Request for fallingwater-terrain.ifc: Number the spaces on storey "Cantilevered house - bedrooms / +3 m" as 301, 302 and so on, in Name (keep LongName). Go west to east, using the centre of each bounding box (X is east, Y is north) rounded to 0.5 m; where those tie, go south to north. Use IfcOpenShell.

First a look at what the model holds.

```python
import ifcopenshell
import ifcopenshell.util.element
import ifcopenshell.util.placement

model = ifcopenshell.open("fallingwater-terrain.ifc")
print(model.schema)
storey = next(s for s in model.by_type("IfcBuildingStorey") if s.Name == "Cantilevered house - bedrooms / +3 m")
spaces = [e for e in ifcopenshell.util.element.get_decomposition(storey) if e.is_a("IfcSpace")]
for e in sorted(spaces, key=lambda e: e.id()):
    origin = ifcopenshell.util.placement.get_local_placement(e.ObjectPlacement)[:3, 3]
    print(e.id(), e.Name, e.LongName, origin.round(2) + 0.0, sep=" | ")
```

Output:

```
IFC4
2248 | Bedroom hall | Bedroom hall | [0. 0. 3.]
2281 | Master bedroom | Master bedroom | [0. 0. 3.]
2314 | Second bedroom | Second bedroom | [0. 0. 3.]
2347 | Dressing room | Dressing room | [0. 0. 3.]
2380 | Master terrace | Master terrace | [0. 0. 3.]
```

```python
import ifcopenshell
import ifcopenshell.geom
import ifcopenshell.util.element
import ifcopenshell.util.shape

model = ifcopenshell.open("fallingwater-terrain.ifc")
settings = ifcopenshell.geom.settings()
settings.set("use-world-coords", True)


def centre(element):
    shape = ifcopenshell.geom.create_shape(settings, element)
    return ifcopenshell.util.shape.get_bbox_centroid(shape.geometry)


storey = next(s for s in model.by_type("IfcBuildingStorey") if s.Name == "Cantilevered house - bedrooms / +3 m")
spaces = [e for e in ifcopenshell.util.element.get_decomposition(storey) if e.is_a("IfcSpace")]

# Insertion points can sit at a corner or the storey origin, so sort by the geometry (in metres).
centres = {e: centre(e) for e in spaces}
spaces.sort(key=lambda e: (round(centres[e][0] / 0.5), centres[e][1]))

for i, e in enumerate(spaces, start=1):
    number = f"3{i:02d}"
    e.Name = number
    print(e.id(), number)

model.write("fallingwater-terrain-out.ifc")
```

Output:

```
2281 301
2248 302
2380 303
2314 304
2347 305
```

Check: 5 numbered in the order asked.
